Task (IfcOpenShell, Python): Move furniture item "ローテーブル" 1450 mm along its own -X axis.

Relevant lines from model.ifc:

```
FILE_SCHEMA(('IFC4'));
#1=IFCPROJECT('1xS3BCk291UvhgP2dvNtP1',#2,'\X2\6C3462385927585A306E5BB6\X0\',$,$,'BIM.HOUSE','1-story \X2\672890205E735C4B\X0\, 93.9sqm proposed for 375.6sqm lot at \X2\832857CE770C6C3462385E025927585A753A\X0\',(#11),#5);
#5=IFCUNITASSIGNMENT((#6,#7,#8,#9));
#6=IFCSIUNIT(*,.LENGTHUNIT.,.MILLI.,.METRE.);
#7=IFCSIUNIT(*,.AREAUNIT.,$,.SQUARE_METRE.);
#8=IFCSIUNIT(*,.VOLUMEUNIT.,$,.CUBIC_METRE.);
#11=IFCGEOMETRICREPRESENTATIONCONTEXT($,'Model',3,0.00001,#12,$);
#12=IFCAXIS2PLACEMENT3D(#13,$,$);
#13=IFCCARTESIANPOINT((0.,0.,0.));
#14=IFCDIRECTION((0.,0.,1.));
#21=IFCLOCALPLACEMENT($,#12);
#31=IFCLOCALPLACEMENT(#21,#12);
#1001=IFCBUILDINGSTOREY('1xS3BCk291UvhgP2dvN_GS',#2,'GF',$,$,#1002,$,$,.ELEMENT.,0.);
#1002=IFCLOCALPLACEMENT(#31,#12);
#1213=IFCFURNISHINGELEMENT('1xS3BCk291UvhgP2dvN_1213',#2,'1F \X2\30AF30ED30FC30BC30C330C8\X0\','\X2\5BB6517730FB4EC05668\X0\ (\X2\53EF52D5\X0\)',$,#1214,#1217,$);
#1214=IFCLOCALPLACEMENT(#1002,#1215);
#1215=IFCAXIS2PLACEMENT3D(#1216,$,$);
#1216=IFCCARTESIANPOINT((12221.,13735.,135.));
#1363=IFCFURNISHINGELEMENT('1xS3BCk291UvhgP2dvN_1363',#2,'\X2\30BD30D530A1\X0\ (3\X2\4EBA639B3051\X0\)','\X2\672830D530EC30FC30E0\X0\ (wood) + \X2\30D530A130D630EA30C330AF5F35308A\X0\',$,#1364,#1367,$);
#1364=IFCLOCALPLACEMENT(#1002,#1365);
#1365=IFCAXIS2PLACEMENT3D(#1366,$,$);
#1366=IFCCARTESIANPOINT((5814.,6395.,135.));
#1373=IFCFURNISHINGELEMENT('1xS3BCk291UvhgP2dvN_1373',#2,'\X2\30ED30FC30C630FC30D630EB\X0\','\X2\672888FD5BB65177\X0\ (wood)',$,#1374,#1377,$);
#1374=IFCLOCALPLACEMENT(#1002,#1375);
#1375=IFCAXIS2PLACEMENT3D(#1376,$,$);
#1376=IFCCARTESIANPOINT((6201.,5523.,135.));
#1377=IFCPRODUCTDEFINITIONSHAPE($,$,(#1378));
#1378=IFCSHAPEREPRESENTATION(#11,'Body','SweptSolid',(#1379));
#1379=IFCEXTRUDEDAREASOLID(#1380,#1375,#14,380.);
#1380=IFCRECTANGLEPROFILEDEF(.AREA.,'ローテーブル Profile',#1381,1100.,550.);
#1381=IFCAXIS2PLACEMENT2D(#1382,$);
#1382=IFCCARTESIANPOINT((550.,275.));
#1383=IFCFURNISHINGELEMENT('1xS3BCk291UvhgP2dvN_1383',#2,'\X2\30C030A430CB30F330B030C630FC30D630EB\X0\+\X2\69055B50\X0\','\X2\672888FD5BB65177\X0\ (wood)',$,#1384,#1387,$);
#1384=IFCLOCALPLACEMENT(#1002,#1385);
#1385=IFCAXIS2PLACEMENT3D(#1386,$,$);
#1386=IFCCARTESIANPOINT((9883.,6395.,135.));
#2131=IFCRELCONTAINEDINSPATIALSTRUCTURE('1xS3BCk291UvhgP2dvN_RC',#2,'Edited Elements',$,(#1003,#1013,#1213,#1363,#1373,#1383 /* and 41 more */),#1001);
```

```python
import ifcopenshell
import ifcopenshell.api.geometry
import ifcopenshell.util.placement
import ifcopenshell.util.unit

model = ifcopenshell.open("model.ifc")
unit_scale = ifcopenshell.util.unit.calculate_unit_scale(model)

item = model.by_guid("1xS3BCk291UvhgP2dvN_1373")
matrix = ifcopenshell.util.placement.get_local_placement(item.ObjectPlacement)
matrix[:3, 3] -= matrix[:3, 0] * 1.45 / unit_scale
ifcopenshell.api.geometry.edit_object_placement(model, product=item, matrix=matrix, is_si=False)

print(ifcopenshell.util.placement.get_local_placement(item.ObjectPlacement).round(3) + 0.0)

model.write("model_edited.ifc")
```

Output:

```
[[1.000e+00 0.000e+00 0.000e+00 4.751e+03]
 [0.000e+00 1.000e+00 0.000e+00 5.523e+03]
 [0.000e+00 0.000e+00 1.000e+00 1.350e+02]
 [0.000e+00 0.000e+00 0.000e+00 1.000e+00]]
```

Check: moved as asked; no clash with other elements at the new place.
